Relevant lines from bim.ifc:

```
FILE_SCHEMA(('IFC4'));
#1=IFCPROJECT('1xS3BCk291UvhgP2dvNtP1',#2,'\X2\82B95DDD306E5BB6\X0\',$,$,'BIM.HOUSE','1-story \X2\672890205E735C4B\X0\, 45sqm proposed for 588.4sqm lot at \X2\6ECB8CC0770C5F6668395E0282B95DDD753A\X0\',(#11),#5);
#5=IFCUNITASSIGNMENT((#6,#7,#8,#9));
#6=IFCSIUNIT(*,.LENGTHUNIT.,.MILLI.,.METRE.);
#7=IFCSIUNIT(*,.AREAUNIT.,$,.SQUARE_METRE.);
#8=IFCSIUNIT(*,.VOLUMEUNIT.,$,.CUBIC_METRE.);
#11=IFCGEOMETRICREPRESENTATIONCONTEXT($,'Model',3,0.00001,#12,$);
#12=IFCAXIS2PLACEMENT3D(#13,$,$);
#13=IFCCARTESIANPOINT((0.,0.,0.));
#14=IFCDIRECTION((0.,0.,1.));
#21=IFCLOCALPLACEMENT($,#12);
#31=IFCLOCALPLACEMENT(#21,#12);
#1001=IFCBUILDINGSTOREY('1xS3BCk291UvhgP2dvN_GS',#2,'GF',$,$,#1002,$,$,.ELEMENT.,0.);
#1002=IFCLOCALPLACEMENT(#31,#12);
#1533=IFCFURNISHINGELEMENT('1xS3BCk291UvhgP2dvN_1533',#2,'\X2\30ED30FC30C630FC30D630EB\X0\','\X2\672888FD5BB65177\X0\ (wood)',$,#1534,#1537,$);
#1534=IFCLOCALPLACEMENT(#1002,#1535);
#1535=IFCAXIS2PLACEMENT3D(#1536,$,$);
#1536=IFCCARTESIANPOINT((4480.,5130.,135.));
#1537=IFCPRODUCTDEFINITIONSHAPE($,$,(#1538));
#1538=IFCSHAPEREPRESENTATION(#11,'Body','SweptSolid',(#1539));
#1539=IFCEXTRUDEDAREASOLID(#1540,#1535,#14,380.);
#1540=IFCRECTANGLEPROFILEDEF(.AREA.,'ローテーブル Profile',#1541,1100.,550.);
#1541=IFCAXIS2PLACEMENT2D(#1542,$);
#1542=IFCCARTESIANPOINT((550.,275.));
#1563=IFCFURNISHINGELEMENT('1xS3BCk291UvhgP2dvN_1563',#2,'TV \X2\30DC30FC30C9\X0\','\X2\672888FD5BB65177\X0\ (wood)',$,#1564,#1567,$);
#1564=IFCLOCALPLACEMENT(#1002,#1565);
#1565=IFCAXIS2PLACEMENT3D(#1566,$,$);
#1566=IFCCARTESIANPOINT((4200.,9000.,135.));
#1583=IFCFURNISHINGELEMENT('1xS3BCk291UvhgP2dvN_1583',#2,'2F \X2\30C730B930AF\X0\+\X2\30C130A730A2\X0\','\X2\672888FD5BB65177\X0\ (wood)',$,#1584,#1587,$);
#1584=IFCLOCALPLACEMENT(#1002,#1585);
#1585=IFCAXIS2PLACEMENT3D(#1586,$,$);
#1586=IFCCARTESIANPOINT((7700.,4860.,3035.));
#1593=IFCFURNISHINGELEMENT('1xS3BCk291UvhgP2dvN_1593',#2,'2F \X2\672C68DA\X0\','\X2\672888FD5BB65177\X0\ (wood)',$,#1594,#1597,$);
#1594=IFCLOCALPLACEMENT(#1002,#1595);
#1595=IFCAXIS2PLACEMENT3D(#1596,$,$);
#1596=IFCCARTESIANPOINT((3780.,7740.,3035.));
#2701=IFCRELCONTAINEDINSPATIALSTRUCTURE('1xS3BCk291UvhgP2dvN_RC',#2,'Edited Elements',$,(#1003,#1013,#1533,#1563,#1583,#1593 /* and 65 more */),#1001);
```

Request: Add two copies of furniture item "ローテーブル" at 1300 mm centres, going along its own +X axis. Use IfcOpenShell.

```python
import ifcopenshell
import ifcopenshell.api.geometry
import ifcopenshell.api.root
import ifcopenshell.util.element
import ifcopenshell.util.placement
import ifcopenshell.util.unit

model = ifcopenshell.open("bim.ifc")
unit_scale = ifcopenshell.util.unit.calculate_unit_scale(model)


def reuse_history(source, copy):
    """copy_class also copies each property set's owner history, people and application; keep the originals."""
    for rel in copy.IsDefinedBy:
        if rel.is_a("IfcRelDefinesByProperties") and (history := rel.RelatingPropertyDefinition.OwnerHistory):
            rel.RelatingPropertyDefinition.OwnerHistory = source.OwnerHistory
            ifcopenshell.util.element.remove_deep2(model, history)


source = model.by_id(1533)
base = ifcopenshell.util.placement.get_local_placement(source.ObjectPlacement)
step = base[:3, 0] * 1.3 / unit_scale

for i in range(1, 3):
    copy = ifcopenshell.api.root.copy_class(model, product=source)
    copy.Representation = ifcopenshell.util.element.copy_deep(
        model, source.Representation, exclude=["IfcGeometricRepresentationContext", "IfcRepresentationMap"]
    )
    reuse_history(source, copy)
    matrix = base.copy()
    matrix[:3, 3] += i * step
    print("added at", matrix[:3, 3].round(3) + 0.0)
    ifcopenshell.api.geometry.edit_object_placement(model, product=copy, matrix=matrix, is_si=False)

model.write("bim_edited.ifc")
```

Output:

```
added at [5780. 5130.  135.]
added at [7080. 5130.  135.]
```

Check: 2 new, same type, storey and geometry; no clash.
